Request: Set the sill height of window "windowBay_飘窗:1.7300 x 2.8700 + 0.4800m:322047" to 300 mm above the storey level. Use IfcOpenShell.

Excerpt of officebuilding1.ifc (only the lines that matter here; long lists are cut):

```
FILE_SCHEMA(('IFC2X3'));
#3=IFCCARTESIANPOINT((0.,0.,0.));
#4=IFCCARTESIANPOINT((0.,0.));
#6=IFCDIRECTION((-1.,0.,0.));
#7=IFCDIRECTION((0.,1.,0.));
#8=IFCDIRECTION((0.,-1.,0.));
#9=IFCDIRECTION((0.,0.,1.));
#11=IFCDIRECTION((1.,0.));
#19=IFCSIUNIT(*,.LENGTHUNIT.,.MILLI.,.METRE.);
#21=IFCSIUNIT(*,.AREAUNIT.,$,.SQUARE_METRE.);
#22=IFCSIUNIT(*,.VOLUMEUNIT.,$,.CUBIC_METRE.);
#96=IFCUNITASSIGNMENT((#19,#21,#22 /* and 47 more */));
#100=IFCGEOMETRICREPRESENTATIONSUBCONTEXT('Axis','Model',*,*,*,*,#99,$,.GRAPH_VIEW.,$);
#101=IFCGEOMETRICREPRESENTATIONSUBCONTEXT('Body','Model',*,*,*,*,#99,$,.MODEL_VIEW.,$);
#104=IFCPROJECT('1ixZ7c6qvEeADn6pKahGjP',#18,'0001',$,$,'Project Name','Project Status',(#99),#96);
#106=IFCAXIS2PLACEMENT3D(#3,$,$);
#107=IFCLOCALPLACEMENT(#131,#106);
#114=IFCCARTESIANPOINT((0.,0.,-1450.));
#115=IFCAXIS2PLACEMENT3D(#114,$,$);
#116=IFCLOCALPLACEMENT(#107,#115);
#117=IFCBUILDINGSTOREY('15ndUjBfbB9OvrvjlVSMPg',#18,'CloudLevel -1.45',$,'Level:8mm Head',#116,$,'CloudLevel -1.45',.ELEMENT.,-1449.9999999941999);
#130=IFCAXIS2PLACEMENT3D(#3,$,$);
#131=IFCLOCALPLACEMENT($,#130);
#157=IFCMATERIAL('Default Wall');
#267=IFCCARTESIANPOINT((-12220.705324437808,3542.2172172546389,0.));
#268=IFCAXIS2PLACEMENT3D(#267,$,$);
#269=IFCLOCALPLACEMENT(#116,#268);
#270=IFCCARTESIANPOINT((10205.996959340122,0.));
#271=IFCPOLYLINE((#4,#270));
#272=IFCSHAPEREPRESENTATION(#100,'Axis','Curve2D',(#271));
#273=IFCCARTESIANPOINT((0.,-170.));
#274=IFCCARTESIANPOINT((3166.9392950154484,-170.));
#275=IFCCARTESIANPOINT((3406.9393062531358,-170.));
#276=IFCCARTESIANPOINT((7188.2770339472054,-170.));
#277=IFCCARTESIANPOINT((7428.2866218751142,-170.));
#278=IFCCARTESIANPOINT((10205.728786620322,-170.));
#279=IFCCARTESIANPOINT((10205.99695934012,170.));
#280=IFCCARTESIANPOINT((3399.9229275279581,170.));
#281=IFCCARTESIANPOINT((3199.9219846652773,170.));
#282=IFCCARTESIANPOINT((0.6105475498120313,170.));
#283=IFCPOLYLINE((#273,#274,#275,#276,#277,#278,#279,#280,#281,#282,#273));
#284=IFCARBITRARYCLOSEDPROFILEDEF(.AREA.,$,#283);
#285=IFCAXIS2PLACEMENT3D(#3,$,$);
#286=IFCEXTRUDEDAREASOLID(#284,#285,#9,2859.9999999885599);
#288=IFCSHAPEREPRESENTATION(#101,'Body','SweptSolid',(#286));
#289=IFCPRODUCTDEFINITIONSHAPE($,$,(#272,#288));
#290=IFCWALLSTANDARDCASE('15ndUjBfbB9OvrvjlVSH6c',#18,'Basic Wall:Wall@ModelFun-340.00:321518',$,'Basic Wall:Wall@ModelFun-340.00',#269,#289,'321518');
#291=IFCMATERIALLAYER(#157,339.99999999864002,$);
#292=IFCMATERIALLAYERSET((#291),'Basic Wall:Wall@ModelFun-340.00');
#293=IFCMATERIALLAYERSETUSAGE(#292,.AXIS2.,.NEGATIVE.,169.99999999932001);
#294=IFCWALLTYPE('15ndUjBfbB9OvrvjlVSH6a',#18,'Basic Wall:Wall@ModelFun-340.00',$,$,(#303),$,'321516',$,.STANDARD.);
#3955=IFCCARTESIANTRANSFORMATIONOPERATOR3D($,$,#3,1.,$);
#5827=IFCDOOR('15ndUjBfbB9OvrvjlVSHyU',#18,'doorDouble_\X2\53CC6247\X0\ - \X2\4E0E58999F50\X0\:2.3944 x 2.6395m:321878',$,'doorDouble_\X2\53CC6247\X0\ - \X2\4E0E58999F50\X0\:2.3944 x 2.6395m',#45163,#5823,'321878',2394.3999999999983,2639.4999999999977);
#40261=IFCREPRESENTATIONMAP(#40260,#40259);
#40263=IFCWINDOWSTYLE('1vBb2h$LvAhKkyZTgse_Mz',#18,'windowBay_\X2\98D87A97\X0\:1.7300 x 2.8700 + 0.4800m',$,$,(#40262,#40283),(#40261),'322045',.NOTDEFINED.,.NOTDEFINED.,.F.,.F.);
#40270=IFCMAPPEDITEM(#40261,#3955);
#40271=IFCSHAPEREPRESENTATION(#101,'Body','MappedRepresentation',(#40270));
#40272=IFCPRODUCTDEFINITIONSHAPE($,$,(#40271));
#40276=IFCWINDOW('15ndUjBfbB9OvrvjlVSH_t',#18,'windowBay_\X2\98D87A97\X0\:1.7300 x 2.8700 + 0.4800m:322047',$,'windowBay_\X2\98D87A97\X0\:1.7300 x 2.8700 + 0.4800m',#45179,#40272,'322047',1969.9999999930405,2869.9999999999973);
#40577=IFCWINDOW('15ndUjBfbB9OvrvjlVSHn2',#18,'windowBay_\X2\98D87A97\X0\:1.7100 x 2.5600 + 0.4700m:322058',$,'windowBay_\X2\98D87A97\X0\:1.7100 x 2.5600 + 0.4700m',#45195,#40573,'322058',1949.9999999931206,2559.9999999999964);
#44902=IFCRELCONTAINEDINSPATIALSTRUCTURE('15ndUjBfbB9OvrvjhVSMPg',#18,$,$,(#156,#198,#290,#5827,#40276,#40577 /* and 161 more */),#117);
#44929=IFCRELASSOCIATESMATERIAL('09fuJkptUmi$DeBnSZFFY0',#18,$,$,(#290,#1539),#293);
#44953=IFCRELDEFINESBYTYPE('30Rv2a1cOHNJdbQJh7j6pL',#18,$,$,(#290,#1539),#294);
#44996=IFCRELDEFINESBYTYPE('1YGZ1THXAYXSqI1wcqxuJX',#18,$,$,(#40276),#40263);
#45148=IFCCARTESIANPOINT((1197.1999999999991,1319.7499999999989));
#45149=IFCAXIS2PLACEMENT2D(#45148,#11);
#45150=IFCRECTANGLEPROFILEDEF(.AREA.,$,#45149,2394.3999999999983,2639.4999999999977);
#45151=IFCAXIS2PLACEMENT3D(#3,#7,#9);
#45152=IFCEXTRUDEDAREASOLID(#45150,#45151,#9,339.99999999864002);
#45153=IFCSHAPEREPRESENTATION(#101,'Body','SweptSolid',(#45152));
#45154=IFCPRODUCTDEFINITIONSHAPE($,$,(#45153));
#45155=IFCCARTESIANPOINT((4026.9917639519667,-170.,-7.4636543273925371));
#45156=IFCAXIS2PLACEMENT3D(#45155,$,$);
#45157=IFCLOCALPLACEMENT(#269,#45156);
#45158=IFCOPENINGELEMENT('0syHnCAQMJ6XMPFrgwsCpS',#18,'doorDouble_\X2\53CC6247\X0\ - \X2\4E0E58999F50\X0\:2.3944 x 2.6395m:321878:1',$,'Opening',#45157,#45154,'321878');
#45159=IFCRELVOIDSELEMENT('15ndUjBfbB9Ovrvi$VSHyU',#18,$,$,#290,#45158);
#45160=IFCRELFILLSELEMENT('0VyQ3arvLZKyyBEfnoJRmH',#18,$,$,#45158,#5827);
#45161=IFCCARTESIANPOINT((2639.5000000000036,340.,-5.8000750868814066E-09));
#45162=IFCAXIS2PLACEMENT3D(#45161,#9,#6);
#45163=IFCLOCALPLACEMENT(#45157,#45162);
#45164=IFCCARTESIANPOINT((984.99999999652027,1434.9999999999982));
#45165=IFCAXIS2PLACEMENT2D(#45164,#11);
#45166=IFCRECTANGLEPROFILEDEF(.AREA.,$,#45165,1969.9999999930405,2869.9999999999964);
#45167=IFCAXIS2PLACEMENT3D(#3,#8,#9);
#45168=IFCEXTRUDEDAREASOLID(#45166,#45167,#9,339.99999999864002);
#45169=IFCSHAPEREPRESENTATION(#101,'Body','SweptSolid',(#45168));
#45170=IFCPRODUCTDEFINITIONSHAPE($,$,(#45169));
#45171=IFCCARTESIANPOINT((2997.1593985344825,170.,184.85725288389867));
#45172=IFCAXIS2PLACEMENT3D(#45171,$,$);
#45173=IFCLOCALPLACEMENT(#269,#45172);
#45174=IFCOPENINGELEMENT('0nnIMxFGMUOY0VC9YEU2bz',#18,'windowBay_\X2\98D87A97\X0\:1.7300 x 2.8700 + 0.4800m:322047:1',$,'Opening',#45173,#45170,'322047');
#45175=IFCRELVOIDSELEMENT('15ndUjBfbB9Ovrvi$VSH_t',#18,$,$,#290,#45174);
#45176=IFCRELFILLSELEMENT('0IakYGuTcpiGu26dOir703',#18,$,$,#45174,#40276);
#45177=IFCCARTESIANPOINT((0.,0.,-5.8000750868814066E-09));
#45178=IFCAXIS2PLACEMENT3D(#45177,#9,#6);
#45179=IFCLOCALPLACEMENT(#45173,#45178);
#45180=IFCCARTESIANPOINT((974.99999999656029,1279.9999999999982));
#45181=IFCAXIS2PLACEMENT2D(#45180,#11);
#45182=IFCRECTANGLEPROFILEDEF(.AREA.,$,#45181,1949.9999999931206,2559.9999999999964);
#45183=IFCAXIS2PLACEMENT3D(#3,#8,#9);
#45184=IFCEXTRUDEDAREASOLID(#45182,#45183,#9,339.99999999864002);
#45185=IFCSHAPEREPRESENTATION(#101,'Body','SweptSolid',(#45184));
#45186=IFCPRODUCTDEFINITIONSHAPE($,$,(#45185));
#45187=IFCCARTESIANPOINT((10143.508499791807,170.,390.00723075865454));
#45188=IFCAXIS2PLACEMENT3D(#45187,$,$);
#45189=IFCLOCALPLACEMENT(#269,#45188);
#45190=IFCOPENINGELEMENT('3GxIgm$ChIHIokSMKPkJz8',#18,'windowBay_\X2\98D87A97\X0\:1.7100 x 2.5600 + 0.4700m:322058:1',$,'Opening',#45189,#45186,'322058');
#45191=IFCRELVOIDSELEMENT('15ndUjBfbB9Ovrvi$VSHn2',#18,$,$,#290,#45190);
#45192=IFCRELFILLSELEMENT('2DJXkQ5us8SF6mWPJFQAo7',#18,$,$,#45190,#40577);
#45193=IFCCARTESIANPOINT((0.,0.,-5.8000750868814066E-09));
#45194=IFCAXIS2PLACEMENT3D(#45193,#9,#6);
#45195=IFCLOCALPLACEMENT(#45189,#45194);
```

```python
import numpy as np
import ifcopenshell
import ifcopenshell.api.geometry
import ifcopenshell.geom
import ifcopenshell.util.element
import ifcopenshell.util.placement
import ifcopenshell.util.shape
import ifcopenshell.util.unit

model = ifcopenshell.open("officebuilding1.ifc")
unit_scale = ifcopenshell.util.unit.calculate_unit_scale(model)

window = model.by_guid("15ndUjBfbB9OvrvjlVSH_t")
opening = window.FillsVoids[0].RelatingOpeningElement
storey = ifcopenshell.util.element.get_container(window, ifc_class="IfcBuildingStorey")
level = ifcopenshell.util.placement.get_local_placement(storey.ObjectPlacement)[2, 3]

# The opening's origin need not be at the sill, so measure its lowest point.
shape = ifcopenshell.geom.create_shape(ifcopenshell.geom.settings(), opening)
bottom = ifcopenshell.util.shape.get_shape_bottom_elevation(shape, shape.geometry) / unit_scale
dz = level + 300.0 - bottom

shift = np.array([0.0, 0.0, dz])
# The window is placed relative to its opening, so it follows when the opening moves.
matrix = ifcopenshell.util.placement.get_local_placement(opening.ObjectPlacement)
matrix[:3, 3] += shift
ifcopenshell.api.geometry.edit_object_placement(
    model, product=opening, matrix=matrix, is_si=False, should_transform_children=True
)

print(f"moved by {dz * unit_scale:+.3f} m")

model.write("officebuilding1_v2.ifc")
```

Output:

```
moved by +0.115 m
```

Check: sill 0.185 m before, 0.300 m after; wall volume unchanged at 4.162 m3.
